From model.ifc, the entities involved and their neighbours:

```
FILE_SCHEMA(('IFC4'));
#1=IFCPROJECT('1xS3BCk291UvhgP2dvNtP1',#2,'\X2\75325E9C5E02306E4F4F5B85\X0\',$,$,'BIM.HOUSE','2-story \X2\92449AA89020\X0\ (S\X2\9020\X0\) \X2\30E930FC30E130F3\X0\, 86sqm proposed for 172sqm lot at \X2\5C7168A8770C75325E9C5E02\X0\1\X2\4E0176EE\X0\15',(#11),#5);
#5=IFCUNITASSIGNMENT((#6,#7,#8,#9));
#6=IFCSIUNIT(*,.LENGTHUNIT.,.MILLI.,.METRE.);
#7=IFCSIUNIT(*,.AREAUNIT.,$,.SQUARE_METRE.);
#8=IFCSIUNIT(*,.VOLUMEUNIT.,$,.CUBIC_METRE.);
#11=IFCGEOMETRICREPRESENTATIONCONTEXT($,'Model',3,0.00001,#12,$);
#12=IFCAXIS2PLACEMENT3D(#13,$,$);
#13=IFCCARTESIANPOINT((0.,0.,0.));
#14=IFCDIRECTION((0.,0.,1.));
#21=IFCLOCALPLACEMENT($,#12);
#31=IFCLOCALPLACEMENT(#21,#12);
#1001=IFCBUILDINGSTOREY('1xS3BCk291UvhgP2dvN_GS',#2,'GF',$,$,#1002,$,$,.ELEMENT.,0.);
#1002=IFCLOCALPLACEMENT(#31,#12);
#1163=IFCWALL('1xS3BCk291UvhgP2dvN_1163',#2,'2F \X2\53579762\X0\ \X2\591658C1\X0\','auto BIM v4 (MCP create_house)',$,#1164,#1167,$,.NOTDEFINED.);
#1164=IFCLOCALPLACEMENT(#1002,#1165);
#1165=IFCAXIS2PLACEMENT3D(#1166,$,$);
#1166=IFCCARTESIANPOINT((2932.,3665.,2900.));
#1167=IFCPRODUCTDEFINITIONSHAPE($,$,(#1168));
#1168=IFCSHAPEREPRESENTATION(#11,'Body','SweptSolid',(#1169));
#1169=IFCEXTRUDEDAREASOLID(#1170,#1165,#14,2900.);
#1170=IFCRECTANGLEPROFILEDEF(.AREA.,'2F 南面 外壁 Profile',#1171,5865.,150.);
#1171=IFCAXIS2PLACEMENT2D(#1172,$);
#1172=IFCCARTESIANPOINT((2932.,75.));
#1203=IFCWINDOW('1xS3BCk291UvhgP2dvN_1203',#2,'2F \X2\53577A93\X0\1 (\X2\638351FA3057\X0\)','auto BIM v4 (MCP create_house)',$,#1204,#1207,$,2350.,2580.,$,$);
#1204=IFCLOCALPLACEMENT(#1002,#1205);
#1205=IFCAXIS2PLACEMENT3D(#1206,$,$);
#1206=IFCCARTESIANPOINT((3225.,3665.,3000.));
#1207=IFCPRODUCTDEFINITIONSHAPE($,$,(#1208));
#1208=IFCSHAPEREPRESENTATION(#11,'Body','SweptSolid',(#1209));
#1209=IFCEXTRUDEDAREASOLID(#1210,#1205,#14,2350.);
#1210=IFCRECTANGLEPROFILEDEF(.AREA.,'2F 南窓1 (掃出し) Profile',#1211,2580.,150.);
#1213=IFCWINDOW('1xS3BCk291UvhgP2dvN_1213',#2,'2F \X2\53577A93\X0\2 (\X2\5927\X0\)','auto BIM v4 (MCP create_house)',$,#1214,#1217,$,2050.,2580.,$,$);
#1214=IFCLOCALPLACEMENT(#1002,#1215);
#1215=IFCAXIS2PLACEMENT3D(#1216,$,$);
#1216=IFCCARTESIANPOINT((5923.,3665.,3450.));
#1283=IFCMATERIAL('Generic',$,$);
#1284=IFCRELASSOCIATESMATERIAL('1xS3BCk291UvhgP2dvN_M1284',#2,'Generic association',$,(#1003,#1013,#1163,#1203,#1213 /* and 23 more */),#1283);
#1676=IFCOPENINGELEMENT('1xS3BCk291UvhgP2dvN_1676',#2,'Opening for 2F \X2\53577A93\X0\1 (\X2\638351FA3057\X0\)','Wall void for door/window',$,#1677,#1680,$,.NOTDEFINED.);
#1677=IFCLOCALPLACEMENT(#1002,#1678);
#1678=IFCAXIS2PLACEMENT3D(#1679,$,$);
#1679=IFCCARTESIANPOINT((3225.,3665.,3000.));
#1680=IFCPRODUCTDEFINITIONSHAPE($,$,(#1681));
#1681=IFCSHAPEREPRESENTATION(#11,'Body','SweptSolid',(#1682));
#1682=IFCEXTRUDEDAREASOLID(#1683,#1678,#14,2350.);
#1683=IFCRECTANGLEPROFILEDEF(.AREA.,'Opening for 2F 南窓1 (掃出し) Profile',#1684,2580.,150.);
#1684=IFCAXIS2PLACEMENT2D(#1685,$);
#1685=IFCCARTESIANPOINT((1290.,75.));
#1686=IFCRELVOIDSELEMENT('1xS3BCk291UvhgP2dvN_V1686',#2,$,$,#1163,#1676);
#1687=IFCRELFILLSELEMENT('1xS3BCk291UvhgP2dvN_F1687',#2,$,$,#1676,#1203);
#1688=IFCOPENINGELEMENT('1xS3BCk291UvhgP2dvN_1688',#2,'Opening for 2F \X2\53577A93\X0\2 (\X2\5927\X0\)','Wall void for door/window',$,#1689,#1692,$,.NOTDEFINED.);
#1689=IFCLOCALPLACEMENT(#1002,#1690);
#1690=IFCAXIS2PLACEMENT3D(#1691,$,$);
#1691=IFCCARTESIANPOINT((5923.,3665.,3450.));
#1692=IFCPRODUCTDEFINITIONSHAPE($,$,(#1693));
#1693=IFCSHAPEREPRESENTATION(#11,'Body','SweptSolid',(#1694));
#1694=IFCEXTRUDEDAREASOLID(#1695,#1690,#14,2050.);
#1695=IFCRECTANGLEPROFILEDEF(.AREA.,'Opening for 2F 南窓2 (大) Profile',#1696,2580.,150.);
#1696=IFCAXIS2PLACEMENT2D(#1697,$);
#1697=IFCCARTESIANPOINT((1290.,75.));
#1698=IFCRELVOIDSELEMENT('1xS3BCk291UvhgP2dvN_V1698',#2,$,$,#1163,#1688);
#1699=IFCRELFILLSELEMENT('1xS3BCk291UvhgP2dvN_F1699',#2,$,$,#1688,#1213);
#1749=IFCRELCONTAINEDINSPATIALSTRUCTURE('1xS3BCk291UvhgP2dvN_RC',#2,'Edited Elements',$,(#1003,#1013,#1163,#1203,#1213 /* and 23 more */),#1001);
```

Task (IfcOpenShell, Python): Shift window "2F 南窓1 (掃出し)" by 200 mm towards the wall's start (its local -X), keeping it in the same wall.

```python
import ifcopenshell
import ifcopenshell.api.geometry
import ifcopenshell.util.placement
import ifcopenshell.util.unit

model = ifcopenshell.open("model.ifc")
unit_scale = ifcopenshell.util.unit.calculate_unit_scale(model)

window = model.by_guid("1xS3BCk291UvhgP2dvN_1203")
opening = window.FillsVoids[0].RelatingOpeningElement
wall = opening.VoidsElements[0].RelatingBuildingElement

wall_matrix = ifcopenshell.util.placement.get_local_placement(wall.ObjectPlacement)
shift = wall_matrix[:3, 0] * -0.2 / unit_scale
before = ifcopenshell.util.placement.get_local_placement(window.ObjectPlacement)[:3, 3].copy()

# The window is not placed relative to its opening, so move both.
for product in (opening, window):
    matrix = ifcopenshell.util.placement.get_local_placement(product.ObjectPlacement)
    matrix[:3, 3] += shift
    ifcopenshell.api.geometry.edit_object_placement(model, product=product, matrix=matrix, is_si=False)

after = ifcopenshell.util.placement.get_local_placement(window.ObjectPlacement)[:3, 3]
print("window moved by", (after - before).round(3) + 0.0)

model.write("model_v2.ifc")
```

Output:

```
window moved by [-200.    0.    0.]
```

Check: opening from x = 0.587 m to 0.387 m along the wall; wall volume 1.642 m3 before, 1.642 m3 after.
